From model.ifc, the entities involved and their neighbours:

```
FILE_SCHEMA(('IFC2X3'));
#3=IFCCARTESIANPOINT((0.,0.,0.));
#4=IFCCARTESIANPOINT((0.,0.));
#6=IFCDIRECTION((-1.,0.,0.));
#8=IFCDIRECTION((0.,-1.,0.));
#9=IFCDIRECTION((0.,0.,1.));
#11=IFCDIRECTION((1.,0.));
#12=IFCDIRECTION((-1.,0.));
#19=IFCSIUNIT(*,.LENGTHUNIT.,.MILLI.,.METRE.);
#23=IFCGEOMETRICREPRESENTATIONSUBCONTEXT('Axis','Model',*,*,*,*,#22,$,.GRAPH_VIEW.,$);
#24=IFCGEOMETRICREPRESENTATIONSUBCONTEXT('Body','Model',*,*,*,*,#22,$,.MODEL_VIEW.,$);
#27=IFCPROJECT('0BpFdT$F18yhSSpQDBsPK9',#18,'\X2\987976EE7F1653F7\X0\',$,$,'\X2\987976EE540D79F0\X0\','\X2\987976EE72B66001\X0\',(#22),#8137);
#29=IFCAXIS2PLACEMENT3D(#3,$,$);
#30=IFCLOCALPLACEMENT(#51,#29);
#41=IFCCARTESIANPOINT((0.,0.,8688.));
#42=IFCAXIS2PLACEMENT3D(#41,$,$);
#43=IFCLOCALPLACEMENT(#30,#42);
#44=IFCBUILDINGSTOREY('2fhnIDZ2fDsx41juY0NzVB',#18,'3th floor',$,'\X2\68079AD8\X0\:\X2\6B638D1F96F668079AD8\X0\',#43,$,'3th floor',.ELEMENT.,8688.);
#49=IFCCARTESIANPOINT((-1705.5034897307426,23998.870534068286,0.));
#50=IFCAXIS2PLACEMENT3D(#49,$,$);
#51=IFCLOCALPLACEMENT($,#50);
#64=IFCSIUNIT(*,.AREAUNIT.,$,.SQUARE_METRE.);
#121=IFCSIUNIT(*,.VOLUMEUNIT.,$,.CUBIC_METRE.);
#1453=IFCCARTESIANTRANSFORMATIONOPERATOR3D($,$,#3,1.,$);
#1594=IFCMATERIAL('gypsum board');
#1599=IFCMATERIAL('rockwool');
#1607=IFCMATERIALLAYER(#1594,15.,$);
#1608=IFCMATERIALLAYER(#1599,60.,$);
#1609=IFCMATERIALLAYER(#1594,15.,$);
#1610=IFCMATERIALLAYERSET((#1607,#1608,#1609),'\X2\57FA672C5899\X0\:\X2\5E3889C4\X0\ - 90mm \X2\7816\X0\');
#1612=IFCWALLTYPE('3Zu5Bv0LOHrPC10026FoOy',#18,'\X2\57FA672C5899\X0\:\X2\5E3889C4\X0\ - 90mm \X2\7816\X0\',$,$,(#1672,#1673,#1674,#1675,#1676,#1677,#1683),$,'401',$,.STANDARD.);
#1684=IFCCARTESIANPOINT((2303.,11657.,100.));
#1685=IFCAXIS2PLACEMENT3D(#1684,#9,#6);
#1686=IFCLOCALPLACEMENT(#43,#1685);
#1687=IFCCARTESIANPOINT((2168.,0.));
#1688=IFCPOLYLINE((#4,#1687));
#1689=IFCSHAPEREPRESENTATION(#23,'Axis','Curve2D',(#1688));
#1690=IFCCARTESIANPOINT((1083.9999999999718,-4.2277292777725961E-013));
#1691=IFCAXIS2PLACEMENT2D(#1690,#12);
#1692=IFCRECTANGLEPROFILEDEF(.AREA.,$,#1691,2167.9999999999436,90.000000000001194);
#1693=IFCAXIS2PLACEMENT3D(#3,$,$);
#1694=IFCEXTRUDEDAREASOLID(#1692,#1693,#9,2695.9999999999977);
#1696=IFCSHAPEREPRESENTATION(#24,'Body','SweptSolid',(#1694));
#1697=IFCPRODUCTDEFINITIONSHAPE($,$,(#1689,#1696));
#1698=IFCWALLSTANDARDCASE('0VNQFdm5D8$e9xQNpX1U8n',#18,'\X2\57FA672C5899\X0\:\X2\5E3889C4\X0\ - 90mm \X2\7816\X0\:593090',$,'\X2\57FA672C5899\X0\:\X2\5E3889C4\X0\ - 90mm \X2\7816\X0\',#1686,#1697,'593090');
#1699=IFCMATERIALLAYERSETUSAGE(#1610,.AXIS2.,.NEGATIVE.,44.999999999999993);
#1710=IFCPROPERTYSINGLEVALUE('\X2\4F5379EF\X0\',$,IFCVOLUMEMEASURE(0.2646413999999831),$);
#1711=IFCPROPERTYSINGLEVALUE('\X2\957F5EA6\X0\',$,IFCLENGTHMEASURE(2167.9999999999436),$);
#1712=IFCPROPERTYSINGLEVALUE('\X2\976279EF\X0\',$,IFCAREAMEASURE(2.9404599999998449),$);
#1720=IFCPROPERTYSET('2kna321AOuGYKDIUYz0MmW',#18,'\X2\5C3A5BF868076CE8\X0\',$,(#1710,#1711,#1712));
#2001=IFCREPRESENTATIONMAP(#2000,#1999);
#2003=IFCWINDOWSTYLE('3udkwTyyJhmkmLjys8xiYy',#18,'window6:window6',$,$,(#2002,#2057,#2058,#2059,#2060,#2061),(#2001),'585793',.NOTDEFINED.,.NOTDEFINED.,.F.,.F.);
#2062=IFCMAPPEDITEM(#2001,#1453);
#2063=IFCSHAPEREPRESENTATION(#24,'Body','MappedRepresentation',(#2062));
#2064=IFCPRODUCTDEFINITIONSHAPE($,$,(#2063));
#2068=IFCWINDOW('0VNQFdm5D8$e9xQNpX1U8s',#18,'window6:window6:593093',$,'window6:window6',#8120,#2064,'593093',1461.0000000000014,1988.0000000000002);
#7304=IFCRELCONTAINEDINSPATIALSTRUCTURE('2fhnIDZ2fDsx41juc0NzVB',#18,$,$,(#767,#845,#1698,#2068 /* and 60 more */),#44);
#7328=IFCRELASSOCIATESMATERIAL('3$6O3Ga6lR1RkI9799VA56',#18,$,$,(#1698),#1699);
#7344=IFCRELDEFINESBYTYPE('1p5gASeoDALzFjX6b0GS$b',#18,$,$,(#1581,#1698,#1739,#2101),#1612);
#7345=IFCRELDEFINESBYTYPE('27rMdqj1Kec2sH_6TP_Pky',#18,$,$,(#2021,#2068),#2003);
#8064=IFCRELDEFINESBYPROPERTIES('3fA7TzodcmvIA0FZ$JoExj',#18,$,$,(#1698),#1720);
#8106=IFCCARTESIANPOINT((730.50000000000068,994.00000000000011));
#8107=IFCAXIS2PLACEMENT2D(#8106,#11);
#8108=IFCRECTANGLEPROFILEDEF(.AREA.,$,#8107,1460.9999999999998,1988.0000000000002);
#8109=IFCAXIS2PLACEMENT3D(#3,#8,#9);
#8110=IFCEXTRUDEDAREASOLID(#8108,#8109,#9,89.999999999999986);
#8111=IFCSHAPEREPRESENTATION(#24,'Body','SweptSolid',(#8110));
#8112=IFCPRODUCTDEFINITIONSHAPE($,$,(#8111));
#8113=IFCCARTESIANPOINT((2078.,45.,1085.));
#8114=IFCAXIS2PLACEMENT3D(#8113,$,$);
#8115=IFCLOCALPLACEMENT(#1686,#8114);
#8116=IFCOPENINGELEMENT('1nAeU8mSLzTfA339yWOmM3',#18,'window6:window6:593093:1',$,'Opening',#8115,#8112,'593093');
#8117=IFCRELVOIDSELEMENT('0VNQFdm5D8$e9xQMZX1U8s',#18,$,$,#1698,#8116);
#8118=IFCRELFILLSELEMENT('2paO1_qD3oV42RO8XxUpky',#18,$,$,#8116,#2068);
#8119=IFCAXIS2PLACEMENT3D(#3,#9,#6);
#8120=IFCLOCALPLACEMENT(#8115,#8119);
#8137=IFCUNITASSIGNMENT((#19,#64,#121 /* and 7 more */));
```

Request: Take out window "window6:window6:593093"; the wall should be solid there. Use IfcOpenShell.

```python
import ifcopenshell
import ifcopenshell.api.feature
import ifcopenshell.api.pset
import ifcopenshell.api.root
import ifcopenshell.geom
import ifcopenshell.util.element
import ifcopenshell.util.shape
import ifcopenshell.util.unit

model = ifcopenshell.open("model.ifc")
area_scale = ifcopenshell.util.unit.calculate_unit_scale(model, "AREAUNIT")
volume_scale = ifcopenshell.util.unit.calculate_unit_scale(model, "VOLUMEUNIT")
settings = ifcopenshell.geom.settings()


def volume(element):
    """Net volume in cubic metres, openings subtracted."""
    shape = ifcopenshell.geom.create_shape(settings, element)
    return ifcopenshell.util.shape.get_volume(shape.geometry)


window = model.by_guid("0VNQFdm5D8$e9xQNpX1U8s")
opening = window.FillsVoids[0].RelatingOpeningElement
wall = opening.VoidsElements[0].RelatingBuildingElement
before = volume(wall)

ifcopenshell.api.root.remove_product(model, product=window)
ifcopenshell.api.feature.remove_feature(model, feature=opening)

after = volume(wall)
thickness = 0.09  # wall thickness in metres

# Update the wall's stored quantities.
pset = model.by_id(ifcopenshell.util.element.get_pset(wall, "尺寸标注", should_inherit=False)["id"])
ifcopenshell.api.pset.edit_pset(model, pset=pset, properties={
    "体积": model.create_entity("IfcVolumeMeasure", after / volume_scale),
    "面积": model.create_entity("IfcAreaMeasure", after / thickness / area_scale),
})

print(f"wall volume {before:.3f} -> {after:.3f} m3")

model.write("model-out.ifc")
```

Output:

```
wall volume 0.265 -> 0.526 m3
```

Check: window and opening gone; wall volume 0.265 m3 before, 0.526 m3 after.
